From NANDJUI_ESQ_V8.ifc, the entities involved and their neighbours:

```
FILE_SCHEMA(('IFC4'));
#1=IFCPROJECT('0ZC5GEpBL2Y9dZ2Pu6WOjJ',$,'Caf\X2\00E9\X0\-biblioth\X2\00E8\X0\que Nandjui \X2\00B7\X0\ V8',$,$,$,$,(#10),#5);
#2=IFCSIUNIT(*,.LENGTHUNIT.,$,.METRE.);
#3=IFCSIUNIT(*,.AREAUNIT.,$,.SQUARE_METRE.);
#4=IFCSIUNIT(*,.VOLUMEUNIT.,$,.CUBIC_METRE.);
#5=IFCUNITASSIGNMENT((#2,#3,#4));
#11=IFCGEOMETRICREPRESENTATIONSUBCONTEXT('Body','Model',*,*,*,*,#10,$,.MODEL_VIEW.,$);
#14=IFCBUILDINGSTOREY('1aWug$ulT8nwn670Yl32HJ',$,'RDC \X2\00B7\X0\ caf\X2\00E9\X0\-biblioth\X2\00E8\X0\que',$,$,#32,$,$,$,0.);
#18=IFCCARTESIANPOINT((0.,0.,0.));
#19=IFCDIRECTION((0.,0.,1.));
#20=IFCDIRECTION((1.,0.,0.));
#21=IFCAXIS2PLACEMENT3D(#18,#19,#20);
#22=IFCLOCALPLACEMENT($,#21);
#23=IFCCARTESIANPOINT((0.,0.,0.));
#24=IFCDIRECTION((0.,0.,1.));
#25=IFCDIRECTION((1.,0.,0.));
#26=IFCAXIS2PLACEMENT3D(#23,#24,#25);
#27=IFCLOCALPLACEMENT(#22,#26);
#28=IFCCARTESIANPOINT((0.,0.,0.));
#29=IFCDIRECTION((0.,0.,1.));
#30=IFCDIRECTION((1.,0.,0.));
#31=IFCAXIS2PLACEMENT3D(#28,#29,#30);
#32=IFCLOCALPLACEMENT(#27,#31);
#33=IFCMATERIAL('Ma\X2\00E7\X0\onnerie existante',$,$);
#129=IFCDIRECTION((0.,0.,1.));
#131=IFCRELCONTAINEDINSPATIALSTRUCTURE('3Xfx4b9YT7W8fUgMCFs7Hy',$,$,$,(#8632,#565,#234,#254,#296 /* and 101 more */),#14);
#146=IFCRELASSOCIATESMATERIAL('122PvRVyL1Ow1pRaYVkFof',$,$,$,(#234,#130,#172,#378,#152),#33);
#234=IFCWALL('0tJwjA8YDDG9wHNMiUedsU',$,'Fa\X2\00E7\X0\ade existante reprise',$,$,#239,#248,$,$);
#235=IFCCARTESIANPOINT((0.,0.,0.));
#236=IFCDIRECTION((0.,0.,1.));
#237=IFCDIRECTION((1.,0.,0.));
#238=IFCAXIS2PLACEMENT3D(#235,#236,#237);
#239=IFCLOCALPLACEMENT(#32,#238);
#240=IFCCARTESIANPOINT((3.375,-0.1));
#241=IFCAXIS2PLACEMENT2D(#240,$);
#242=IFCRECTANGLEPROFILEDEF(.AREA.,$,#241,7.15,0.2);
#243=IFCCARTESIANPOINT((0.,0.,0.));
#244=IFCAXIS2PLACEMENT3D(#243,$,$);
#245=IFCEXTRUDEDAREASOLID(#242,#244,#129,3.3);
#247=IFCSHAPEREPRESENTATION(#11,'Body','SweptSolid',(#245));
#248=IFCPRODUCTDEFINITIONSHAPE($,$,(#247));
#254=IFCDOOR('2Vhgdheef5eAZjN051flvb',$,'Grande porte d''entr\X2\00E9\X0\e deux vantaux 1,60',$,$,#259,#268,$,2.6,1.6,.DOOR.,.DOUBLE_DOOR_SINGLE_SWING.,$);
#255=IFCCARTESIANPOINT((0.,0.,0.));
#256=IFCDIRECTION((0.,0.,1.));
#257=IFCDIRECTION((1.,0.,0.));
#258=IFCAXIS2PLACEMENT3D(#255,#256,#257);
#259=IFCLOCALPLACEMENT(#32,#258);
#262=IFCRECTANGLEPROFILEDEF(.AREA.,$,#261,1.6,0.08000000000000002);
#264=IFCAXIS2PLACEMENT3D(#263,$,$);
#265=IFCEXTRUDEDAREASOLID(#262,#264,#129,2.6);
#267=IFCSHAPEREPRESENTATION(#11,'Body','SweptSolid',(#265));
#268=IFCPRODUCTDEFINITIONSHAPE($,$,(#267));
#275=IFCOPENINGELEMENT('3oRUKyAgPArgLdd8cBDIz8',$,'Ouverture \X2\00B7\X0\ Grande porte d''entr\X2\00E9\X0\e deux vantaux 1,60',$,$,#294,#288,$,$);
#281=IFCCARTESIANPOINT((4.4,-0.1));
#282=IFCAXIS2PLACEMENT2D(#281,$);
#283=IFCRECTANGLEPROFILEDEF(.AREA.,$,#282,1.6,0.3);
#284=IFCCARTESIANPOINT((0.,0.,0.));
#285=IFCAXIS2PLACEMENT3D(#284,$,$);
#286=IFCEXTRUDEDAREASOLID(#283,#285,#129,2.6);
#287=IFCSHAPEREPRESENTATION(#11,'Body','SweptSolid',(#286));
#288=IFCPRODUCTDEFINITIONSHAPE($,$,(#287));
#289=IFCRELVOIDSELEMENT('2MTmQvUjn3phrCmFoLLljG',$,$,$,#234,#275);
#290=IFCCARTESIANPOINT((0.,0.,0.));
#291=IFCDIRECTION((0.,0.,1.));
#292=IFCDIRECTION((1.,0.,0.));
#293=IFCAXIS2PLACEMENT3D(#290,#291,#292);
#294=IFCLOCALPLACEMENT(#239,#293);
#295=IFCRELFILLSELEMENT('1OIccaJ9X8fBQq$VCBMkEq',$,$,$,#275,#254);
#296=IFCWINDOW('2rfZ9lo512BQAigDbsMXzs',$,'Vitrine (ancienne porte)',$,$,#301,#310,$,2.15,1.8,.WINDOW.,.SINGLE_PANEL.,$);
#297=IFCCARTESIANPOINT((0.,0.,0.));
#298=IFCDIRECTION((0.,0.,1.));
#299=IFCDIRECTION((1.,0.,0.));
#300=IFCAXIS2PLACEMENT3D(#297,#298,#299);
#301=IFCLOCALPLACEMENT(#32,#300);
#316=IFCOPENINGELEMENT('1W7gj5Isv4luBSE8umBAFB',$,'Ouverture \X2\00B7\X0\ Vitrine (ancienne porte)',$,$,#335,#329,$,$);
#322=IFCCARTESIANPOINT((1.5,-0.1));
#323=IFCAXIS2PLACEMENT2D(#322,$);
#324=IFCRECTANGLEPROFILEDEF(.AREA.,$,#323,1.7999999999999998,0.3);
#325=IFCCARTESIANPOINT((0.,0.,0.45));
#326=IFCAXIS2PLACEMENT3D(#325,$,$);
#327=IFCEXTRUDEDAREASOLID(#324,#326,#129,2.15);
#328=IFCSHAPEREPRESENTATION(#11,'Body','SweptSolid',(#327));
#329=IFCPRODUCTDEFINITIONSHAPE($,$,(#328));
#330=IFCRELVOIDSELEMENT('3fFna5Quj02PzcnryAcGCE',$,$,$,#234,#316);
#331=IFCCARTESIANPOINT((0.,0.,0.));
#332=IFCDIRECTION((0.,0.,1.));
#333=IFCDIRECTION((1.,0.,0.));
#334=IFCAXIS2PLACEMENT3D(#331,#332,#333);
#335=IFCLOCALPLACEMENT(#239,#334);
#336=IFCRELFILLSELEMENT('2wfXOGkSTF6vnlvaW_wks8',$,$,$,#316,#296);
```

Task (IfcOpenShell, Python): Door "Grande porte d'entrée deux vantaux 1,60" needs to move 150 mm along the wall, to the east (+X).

```python
import ifcopenshell
import ifcopenshell.api.geometry
import ifcopenshell.util.placement
import ifcopenshell.util.unit

model = ifcopenshell.open("NANDJUI_ESQ_V8.ifc")
unit_scale = ifcopenshell.util.unit.calculate_unit_scale(model)

door = model.by_guid("2Vhgdheef5eAZjN051flvb")
opening = door.FillsVoids[0].RelatingOpeningElement
wall = opening.VoidsElements[0].RelatingBuildingElement

wall_matrix = ifcopenshell.util.placement.get_local_placement(wall.ObjectPlacement)
shift = wall_matrix[:3, 0] * 0.15 / unit_scale
before = ifcopenshell.util.placement.get_local_placement(door.ObjectPlacement)[:3, 3].copy()

# The door is not placed relative to its opening, so move both.
for product in (opening, door):
    matrix = ifcopenshell.util.placement.get_local_placement(product.ObjectPlacement)
    matrix[:3, 3] += shift
    ifcopenshell.api.geometry.edit_object_placement(model, product=product, matrix=matrix, is_si=False)

after = ifcopenshell.util.placement.get_local_placement(door.ObjectPlacement)[:3, 3]
print("door moved by", (after - before).round(3) + 0.0)

model.write("NANDJUI_ESQ_V8_updated.ifc")
```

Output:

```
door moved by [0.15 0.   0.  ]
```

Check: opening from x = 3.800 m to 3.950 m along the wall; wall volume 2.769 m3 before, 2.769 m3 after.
